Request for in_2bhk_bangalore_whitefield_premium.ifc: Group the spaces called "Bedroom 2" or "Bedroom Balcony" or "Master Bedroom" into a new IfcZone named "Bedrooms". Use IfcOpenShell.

First a look at what the model holds.

```python
import ifcopenshell

model = ifcopenshell.open("in_2bhk_bangalore_whitefield_premium.ifc")
print(model.schema)
seen = {}
for space in model.by_type("IfcSpace"):
    seen[space.LongName] = seen.get(space.LongName, 0) + 1
for name, count in sorted(seen.items(), key=str):
    print(count, "x", name)
print("zones:", [z.Name for z in model.by_type("IfcZone")][:20])
```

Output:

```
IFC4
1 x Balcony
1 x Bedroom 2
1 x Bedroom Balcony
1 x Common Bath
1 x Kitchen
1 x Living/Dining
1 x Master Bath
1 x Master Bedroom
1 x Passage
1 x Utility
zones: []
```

```python
import ifcopenshell
import ifcopenshell.api.group
import ifcopenshell.api.root

model = ifcopenshell.open("in_2bhk_bangalore_whitefield_premium.ifc")

names = {"Bedroom 2", "Bedroom Balcony", "Master Bedroom"}
spaces = [s for s in model.by_type("IfcSpace") if s.LongName in names]

zone = ifcopenshell.api.root.create_entity(model, ifc_class="IfcZone", name="Bedrooms")
ifcopenshell.api.group.assign_group(model, products=spaces, group=zone)
print(len(spaces), "spaces in", zone.Name)

model.write("in_2bhk_bangalore_whitefield_premium_rev.ifc")
```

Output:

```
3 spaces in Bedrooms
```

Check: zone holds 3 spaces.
